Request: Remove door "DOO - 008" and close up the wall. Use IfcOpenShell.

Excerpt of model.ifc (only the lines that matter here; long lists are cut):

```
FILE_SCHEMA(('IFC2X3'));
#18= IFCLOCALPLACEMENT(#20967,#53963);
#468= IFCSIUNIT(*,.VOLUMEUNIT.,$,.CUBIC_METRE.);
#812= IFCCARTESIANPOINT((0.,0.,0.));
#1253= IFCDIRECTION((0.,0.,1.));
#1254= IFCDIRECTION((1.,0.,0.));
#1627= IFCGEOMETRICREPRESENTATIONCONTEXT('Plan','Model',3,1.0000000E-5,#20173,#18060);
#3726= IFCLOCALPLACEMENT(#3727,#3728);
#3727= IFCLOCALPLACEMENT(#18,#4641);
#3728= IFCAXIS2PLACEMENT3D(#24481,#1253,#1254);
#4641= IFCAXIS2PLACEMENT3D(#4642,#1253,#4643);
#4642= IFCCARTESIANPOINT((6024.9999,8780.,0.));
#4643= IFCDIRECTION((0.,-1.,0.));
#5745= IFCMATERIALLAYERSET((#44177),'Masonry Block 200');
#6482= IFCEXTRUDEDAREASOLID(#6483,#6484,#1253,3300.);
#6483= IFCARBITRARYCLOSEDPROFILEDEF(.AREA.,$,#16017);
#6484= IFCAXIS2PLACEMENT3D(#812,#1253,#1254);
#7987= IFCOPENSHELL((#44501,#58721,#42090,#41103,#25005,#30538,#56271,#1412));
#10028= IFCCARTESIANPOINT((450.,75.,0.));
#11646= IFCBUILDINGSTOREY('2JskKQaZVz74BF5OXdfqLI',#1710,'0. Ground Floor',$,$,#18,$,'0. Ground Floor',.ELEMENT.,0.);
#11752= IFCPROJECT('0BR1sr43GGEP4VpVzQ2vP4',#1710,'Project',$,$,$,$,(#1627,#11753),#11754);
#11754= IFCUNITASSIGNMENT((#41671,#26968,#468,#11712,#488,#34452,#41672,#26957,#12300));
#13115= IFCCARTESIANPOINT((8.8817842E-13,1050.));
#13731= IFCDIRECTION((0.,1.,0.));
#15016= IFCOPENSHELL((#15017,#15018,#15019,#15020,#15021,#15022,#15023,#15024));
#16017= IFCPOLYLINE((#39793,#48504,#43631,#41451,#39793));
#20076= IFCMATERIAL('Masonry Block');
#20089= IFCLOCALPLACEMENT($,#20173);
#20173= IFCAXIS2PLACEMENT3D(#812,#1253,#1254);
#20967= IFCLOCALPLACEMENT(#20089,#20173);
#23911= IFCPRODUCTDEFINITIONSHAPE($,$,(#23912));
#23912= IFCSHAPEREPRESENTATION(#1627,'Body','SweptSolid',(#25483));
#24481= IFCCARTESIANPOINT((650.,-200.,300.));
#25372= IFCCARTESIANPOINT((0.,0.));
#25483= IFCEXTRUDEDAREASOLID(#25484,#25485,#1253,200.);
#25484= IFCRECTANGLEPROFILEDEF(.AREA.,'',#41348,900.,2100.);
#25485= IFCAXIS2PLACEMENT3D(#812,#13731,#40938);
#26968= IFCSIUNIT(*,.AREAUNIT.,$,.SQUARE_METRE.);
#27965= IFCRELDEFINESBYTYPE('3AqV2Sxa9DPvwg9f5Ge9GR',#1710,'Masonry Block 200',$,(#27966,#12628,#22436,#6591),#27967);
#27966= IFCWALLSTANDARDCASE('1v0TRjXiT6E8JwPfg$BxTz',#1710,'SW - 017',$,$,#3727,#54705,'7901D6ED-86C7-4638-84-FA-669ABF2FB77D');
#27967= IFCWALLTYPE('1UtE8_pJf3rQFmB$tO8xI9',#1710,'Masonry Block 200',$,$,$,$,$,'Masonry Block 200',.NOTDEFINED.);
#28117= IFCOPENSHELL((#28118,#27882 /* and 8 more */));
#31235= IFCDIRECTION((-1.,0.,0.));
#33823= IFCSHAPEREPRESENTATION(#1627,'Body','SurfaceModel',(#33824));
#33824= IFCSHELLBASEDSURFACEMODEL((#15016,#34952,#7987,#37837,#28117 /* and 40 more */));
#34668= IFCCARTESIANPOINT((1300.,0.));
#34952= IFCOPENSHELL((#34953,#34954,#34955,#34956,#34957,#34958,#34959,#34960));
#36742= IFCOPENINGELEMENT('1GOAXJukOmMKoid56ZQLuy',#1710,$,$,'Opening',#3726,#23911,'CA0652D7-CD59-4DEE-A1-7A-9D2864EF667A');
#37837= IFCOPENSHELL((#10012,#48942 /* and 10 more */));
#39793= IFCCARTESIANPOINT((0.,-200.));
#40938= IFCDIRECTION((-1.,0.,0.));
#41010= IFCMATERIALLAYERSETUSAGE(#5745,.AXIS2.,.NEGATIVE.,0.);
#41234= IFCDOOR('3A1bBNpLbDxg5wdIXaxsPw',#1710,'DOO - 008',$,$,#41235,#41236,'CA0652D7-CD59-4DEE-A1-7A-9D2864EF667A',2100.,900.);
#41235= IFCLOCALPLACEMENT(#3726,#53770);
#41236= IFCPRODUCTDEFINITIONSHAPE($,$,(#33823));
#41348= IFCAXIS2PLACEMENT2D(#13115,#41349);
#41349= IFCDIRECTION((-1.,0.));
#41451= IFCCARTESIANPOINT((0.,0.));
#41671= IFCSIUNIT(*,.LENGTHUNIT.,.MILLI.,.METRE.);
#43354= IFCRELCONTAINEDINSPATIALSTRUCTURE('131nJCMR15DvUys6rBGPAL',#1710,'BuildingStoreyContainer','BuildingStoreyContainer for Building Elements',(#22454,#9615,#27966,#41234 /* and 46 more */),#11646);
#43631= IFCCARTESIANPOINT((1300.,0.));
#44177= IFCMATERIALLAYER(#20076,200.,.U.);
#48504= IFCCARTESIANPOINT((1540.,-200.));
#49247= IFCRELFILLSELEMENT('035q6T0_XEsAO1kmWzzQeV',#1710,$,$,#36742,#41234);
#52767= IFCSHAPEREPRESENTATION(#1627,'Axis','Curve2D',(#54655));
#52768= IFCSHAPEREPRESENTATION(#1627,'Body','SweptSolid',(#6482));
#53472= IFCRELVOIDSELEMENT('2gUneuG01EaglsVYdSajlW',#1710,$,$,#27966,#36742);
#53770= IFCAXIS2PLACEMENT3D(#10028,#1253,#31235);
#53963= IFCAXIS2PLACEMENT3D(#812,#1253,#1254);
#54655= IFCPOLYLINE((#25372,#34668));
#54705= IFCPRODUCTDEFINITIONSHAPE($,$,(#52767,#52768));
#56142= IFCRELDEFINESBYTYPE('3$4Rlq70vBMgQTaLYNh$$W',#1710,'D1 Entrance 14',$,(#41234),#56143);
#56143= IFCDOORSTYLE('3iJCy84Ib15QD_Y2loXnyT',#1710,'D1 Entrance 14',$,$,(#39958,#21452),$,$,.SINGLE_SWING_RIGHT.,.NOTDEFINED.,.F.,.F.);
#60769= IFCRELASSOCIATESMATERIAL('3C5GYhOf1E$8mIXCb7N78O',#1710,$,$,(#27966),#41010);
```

```python
import ifcopenshell
import ifcopenshell.api.feature
import ifcopenshell.api.root
import ifcopenshell.geom
import ifcopenshell.util.shape

model = ifcopenshell.open("model.ifc")
settings = ifcopenshell.geom.settings()


def volume(element):
    """Net volume in cubic metres, openings subtracted."""
    shape = ifcopenshell.geom.create_shape(settings, element)
    return ifcopenshell.util.shape.get_volume(shape.geometry)


door = model.by_guid("3A1bBNpLbDxg5wdIXaxsPw")
opening = door.FillsVoids[0].RelatingOpeningElement
wall = opening.VoidsElements[0].RelatingBuildingElement
before = volume(wall)

ifcopenshell.api.root.remove_product(model, product=door)
ifcopenshell.api.feature.remove_feature(model, feature=opening)

after = volume(wall)

print(f"wall volume {before:.3f} -> {after:.3f} m3")

model.write("model_v2.ifc")
```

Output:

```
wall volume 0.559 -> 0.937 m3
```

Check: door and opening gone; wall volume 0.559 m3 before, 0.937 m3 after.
